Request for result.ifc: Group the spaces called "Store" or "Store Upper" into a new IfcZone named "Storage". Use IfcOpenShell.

First a look at what the model holds.

```python
import ifcopenshell

model = ifcopenshell.open("result.ifc")
print(model.schema)
seen = {}
for space in model.by_type("IfcSpace"):
    seen[space.LongName] = seen.get(space.LongName, 0) + 1
for name, count in sorted(seen.items(), key=str):
    print(count, "x", name)
print("zones:", [z.Name for z in model.by_type("IfcZone")][:20])
```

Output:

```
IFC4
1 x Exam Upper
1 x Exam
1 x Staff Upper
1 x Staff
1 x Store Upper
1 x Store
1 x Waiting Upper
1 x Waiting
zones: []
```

```python
import ifcopenshell
import ifcopenshell.api.group
import ifcopenshell.api.root

model = ifcopenshell.open("result.ifc")

names = {"Store", "Store Upper"}
spaces = [s for s in model.by_type("IfcSpace") if s.LongName in names]

zone = ifcopenshell.api.root.create_entity(model, ifc_class="IfcZone", name="Storage")
ifcopenshell.api.group.assign_group(model, products=spaces, group=zone)
print(len(spaces), "spaces in", zone.Name)

model.write("result_updated.ifc")
```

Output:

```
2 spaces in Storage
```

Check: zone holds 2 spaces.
